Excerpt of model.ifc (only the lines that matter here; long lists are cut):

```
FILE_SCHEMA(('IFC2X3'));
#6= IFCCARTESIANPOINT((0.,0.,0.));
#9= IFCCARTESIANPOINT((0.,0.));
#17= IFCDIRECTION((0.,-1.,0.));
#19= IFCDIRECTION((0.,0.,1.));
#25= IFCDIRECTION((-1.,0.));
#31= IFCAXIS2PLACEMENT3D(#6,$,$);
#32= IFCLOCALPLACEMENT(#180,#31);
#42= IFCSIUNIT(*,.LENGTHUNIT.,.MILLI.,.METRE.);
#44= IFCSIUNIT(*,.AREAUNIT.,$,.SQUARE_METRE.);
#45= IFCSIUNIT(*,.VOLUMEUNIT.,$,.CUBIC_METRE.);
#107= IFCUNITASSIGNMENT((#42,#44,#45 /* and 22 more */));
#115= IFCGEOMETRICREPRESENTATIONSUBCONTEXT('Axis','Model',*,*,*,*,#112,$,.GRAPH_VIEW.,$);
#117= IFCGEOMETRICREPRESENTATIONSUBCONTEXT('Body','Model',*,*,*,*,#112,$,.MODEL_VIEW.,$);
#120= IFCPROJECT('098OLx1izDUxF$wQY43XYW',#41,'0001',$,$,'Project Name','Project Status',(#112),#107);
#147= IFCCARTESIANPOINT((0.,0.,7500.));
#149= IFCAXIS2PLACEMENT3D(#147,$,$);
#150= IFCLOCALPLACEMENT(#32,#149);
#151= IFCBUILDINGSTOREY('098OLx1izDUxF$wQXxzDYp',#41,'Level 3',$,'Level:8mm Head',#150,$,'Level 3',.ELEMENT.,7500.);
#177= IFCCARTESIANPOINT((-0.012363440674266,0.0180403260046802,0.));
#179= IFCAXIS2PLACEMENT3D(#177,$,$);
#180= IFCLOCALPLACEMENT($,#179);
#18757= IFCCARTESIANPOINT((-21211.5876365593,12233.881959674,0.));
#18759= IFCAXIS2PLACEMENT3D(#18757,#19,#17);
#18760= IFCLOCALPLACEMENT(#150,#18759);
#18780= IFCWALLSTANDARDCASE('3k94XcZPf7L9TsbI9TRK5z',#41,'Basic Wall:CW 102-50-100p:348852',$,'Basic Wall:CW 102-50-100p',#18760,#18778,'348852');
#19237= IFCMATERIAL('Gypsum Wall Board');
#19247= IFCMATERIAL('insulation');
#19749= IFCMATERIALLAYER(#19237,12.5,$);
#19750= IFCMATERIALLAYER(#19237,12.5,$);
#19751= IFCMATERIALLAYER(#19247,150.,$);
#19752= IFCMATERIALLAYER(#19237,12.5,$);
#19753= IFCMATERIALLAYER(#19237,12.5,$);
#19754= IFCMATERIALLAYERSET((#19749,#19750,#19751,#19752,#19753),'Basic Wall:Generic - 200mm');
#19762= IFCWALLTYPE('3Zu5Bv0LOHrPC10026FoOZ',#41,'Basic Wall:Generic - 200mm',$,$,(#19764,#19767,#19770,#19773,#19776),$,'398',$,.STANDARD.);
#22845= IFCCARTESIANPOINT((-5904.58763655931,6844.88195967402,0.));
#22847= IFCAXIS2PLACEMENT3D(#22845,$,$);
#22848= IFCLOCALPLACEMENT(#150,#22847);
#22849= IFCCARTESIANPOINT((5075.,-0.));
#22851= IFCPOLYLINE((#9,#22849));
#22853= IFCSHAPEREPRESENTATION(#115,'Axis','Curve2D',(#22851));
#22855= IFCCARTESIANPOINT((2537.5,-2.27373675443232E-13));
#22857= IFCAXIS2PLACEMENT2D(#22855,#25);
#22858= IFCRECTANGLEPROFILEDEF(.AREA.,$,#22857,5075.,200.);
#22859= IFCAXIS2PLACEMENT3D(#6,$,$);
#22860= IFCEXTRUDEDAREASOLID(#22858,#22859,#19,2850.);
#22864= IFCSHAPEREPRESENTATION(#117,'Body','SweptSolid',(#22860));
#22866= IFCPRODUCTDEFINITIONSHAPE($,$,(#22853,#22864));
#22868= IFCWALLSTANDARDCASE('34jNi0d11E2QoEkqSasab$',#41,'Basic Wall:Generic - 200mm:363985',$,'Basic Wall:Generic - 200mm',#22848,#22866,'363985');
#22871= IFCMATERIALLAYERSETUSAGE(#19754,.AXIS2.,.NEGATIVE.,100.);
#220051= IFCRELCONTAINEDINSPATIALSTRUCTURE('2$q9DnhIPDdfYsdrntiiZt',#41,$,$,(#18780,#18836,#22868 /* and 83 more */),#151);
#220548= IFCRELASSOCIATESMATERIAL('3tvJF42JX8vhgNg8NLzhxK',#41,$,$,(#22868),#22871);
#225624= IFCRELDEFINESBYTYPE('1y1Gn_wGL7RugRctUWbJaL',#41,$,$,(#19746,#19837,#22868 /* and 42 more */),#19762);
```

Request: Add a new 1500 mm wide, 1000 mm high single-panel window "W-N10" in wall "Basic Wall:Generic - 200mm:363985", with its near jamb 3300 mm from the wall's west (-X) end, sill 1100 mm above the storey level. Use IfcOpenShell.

```python
import numpy as np
import ifcopenshell
import ifcopenshell.api.feature
import ifcopenshell.api.geometry
import ifcopenshell.api.root
import ifcopenshell.api.spatial
import ifcopenshell.api.type
import ifcopenshell.geom
import ifcopenshell.util.element
import ifcopenshell.util.placement
import ifcopenshell.util.representation
import ifcopenshell.util.shape
import ifcopenshell.util.unit

model = ifcopenshell.open("model.ifc")
unit_scale = ifcopenshell.util.unit.calculate_unit_scale(model)
settings = ifcopenshell.geom.settings()


def volume(element):
    """Net volume in cubic metres, openings subtracted."""
    shape = ifcopenshell.geom.create_shape(settings, element)
    return ifcopenshell.util.shape.get_volume(shape.geometry)


wall = model.by_id(22868)
storey = ifcopenshell.util.element.get_container(wall, ifc_class="IfcBuildingStorey")
context = ifcopenshell.util.representation.get_context(model, "Model", "Body", "MODEL_VIEW")
before = volume(wall)

width, height, from_end, sill = 1.5, 1, 3.3, 1.1  # metres

# The wall runs along its own X axis, and the end named is its -X end.
wall_shape = ifcopenshell.geom.create_shape(settings, wall)
x, y, z = ifcopenshell.util.shape.get_vertices(wall_shape.geometry).T
start = x.min() + from_end
face, thickness = float(y.min()), float(y.max() - y.min())
wall_matrix = ifcopenshell.util.placement.get_local_placement(wall.ObjectPlacement)
level = ifcopenshell.util.placement.get_local_placement(storey.ObjectPlacement)[2, 3]


def in_wall(x, y):
    """Placement at x, y metres in the wall's axes, at sill height."""
    matrix = wall_matrix.copy()
    matrix[:, 3] = wall_matrix @ np.array([x / unit_scale, y / unit_scale, 0.0, 1.0])
    matrix[2, 3] = level + sill / unit_scale
    return matrix


# Opening: a box that overshoots both wall faces by 50 mm.
opening = ifcopenshell.api.root.create_entity(model, ifc_class="IfcOpeningElement")
box = ifcopenshell.api.geometry.add_wall_representation(
    model, context=context, length=width, height=height, thickness=thickness + 0.1
)
ifcopenshell.api.geometry.assign_representation(model, product=opening, representation=box)
ifcopenshell.api.geometry.edit_object_placement(model, product=opening, matrix=in_wall(start, face - 0.05), is_si=False)
ifcopenshell.api.feature.add_feature(model, feature=opening, element=wall)

window = ifcopenshell.api.root.create_entity(model, ifc_class="IfcWindow", name="W-N10")
window.OverallWidth, window.OverallHeight = width / unit_scale, height / unit_scale
body = ifcopenshell.api.geometry.add_window_representation(
    model,
    context=context,
    overall_width=window.OverallWidth,
    overall_height=window.OverallHeight,
    partition_type="SINGLE_PANEL",
)
ifcopenshell.api.geometry.assign_representation(model, product=window, representation=body)
ifcopenshell.api.spatial.assign_container(model, products=[window], relating_structure=storey)
fills = ifcopenshell.api.feature.add_filling(model, opening=opening, element=window)
fills.OwnerHistory = window.OwnerHistory  # required in IFC2X3

# IFC2X3 keeps the operation on the window style.
style = ifcopenshell.api.root.create_entity(model, ifc_class="IfcWindowStyle", name="W-N10")
style.OperationType, style.ConstructionType = "SINGLE_PANEL", "NOTDEFINED"
style.ParameterTakesPrecedence = style.Sizeable = False
ifcopenshell.api.type.assign_type(model, related_objects=[window], relating_type=style)

# Centre the window in the wall's thickness.
ifcopenshell.api.geometry.edit_object_placement(model, product=window, matrix=in_wall(start, face), is_si=False)
window_shape = ifcopenshell.geom.create_shape(settings, window)
depth = ifcopenshell.util.shape.get_vertices(window_shape.geometry)[:, 1]
offset = face + thickness / 2 - (depth.min() + depth.max()) / 2
ifcopenshell.api.geometry.edit_object_placement(model, product=window, matrix=in_wall(start, offset), is_si=False)

after = volume(wall)

print(f"wall volume {before:.3f} -> {after:.3f} m3")

model.write("model-out.ifc")
```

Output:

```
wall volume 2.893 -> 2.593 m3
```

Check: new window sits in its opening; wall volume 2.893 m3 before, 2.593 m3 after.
